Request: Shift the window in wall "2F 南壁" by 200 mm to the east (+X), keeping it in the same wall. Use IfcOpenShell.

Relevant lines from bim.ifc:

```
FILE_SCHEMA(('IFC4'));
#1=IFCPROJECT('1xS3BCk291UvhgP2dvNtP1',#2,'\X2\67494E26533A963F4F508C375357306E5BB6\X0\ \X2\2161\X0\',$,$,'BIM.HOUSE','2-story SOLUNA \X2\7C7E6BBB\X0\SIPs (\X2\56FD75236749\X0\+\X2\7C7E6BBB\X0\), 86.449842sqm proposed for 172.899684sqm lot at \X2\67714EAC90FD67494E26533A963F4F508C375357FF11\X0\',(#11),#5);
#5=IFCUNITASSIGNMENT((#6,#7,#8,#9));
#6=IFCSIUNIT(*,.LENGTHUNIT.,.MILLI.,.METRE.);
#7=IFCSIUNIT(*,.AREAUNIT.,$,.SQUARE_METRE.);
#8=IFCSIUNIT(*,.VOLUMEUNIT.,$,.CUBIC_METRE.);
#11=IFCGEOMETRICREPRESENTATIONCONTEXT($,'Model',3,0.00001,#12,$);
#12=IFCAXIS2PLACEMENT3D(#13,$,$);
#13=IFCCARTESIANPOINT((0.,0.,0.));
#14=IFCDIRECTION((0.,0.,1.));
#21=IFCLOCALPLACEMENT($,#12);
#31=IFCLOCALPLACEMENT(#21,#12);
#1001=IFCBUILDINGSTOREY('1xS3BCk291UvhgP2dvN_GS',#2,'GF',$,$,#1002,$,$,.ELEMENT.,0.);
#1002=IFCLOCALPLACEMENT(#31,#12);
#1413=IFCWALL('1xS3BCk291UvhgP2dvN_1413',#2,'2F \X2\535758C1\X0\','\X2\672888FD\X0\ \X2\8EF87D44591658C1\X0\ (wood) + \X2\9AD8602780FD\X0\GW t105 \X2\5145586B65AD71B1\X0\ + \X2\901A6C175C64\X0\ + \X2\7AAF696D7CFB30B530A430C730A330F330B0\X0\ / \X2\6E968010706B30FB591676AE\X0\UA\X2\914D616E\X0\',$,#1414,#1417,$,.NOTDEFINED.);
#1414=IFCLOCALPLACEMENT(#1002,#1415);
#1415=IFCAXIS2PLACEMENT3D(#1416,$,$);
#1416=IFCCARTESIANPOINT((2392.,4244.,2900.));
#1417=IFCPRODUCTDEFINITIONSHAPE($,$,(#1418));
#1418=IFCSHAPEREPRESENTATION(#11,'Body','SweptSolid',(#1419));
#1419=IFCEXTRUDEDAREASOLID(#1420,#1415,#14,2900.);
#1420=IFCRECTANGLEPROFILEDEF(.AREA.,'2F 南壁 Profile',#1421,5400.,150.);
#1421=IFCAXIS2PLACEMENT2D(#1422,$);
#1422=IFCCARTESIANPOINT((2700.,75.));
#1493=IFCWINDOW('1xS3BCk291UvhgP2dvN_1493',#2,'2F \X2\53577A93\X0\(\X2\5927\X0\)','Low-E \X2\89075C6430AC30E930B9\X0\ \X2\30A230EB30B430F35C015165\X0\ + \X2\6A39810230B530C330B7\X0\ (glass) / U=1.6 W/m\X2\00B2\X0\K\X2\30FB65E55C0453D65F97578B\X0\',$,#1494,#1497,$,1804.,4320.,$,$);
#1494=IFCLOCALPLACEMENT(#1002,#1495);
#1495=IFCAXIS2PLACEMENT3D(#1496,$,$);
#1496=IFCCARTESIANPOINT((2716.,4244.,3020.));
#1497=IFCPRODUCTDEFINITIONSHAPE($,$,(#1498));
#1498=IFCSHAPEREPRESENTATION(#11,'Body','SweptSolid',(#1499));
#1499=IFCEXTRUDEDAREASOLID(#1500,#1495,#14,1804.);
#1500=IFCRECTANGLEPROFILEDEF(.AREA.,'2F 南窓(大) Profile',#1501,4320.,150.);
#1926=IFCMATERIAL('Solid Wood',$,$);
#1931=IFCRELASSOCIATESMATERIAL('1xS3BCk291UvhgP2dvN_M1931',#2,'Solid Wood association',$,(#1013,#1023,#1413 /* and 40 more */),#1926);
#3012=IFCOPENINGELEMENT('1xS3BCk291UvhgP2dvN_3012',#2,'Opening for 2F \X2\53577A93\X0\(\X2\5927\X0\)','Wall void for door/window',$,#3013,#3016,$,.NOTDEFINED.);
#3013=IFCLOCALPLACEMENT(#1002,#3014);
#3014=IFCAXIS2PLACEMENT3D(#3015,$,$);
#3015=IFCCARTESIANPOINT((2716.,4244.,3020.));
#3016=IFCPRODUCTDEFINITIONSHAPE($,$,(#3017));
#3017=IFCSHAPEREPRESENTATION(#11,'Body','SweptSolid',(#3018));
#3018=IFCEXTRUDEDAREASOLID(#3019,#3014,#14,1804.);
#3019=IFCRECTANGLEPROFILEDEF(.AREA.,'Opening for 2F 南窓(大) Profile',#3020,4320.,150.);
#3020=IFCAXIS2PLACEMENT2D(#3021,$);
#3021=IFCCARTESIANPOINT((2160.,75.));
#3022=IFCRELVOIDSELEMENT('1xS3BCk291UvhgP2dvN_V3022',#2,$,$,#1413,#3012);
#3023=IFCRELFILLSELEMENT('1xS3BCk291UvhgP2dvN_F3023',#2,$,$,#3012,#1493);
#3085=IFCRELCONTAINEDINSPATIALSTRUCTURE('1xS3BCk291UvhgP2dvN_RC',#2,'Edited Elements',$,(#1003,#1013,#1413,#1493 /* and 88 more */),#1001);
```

```python
import ifcopenshell
import ifcopenshell.api.geometry
import ifcopenshell.util.placement
import ifcopenshell.util.unit

model = ifcopenshell.open("bim.ifc")
unit_scale = ifcopenshell.util.unit.calculate_unit_scale(model)

window = model.by_guid("1xS3BCk291UvhgP2dvN_1493")
opening = window.FillsVoids[0].RelatingOpeningElement
wall = opening.VoidsElements[0].RelatingBuildingElement

wall_matrix = ifcopenshell.util.placement.get_local_placement(wall.ObjectPlacement)
shift = wall_matrix[:3, 0] * 0.2 / unit_scale
before = ifcopenshell.util.placement.get_local_placement(window.ObjectPlacement)[:3, 3].copy()

# The window is not placed relative to its opening, so move both.
for product in (opening, window):
    matrix = ifcopenshell.util.placement.get_local_placement(product.ObjectPlacement)
    matrix[:3, 3] += shift
    ifcopenshell.api.geometry.edit_object_placement(model, product=product, matrix=matrix, is_si=False)

after = ifcopenshell.util.placement.get_local_placement(window.ObjectPlacement)[:3, 3]
print("window moved by", (after - before).round(3) + 0.0)

model.write("bim_edited.ifc")
```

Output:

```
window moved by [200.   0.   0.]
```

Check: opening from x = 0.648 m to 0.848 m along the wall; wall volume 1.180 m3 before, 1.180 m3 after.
